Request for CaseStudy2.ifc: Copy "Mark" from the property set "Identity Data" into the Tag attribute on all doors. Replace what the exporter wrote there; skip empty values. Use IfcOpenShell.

First a look at what the model holds.

```python
import ifcopenshell
import ifcopenshell.util.element

model = ifcopenshell.open("CaseStudy2.ifc")
print(model.schema)
doors = model.by_type("IfcDoor")
print(len(doors), "doors")
for e in doors[:8]:
    source = ifcopenshell.util.element.get_pset(e, "Identity Data", "Mark")
    target = e.Tag
    print(e.id(), repr(source), repr(target), sep=" | ")
```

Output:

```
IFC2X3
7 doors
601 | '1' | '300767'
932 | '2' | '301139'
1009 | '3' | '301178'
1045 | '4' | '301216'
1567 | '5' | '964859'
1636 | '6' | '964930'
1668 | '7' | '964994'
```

```python
import ifcopenshell
import ifcopenshell.util.element

model = ifcopenshell.open("CaseStudy2.ifc")

count = 0
for e in model.by_type("IfcDoor"):
    value = ifcopenshell.util.element.get_pset(e, "Identity Data", "Mark")
    current = e.Tag
    if not value or not value.strip() or current == value:
        continue
    e.Tag = value
    count += 1

print(count, "doors updated")

model.write("CaseStudy2_v2.ifc")
```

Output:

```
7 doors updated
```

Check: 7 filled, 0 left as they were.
